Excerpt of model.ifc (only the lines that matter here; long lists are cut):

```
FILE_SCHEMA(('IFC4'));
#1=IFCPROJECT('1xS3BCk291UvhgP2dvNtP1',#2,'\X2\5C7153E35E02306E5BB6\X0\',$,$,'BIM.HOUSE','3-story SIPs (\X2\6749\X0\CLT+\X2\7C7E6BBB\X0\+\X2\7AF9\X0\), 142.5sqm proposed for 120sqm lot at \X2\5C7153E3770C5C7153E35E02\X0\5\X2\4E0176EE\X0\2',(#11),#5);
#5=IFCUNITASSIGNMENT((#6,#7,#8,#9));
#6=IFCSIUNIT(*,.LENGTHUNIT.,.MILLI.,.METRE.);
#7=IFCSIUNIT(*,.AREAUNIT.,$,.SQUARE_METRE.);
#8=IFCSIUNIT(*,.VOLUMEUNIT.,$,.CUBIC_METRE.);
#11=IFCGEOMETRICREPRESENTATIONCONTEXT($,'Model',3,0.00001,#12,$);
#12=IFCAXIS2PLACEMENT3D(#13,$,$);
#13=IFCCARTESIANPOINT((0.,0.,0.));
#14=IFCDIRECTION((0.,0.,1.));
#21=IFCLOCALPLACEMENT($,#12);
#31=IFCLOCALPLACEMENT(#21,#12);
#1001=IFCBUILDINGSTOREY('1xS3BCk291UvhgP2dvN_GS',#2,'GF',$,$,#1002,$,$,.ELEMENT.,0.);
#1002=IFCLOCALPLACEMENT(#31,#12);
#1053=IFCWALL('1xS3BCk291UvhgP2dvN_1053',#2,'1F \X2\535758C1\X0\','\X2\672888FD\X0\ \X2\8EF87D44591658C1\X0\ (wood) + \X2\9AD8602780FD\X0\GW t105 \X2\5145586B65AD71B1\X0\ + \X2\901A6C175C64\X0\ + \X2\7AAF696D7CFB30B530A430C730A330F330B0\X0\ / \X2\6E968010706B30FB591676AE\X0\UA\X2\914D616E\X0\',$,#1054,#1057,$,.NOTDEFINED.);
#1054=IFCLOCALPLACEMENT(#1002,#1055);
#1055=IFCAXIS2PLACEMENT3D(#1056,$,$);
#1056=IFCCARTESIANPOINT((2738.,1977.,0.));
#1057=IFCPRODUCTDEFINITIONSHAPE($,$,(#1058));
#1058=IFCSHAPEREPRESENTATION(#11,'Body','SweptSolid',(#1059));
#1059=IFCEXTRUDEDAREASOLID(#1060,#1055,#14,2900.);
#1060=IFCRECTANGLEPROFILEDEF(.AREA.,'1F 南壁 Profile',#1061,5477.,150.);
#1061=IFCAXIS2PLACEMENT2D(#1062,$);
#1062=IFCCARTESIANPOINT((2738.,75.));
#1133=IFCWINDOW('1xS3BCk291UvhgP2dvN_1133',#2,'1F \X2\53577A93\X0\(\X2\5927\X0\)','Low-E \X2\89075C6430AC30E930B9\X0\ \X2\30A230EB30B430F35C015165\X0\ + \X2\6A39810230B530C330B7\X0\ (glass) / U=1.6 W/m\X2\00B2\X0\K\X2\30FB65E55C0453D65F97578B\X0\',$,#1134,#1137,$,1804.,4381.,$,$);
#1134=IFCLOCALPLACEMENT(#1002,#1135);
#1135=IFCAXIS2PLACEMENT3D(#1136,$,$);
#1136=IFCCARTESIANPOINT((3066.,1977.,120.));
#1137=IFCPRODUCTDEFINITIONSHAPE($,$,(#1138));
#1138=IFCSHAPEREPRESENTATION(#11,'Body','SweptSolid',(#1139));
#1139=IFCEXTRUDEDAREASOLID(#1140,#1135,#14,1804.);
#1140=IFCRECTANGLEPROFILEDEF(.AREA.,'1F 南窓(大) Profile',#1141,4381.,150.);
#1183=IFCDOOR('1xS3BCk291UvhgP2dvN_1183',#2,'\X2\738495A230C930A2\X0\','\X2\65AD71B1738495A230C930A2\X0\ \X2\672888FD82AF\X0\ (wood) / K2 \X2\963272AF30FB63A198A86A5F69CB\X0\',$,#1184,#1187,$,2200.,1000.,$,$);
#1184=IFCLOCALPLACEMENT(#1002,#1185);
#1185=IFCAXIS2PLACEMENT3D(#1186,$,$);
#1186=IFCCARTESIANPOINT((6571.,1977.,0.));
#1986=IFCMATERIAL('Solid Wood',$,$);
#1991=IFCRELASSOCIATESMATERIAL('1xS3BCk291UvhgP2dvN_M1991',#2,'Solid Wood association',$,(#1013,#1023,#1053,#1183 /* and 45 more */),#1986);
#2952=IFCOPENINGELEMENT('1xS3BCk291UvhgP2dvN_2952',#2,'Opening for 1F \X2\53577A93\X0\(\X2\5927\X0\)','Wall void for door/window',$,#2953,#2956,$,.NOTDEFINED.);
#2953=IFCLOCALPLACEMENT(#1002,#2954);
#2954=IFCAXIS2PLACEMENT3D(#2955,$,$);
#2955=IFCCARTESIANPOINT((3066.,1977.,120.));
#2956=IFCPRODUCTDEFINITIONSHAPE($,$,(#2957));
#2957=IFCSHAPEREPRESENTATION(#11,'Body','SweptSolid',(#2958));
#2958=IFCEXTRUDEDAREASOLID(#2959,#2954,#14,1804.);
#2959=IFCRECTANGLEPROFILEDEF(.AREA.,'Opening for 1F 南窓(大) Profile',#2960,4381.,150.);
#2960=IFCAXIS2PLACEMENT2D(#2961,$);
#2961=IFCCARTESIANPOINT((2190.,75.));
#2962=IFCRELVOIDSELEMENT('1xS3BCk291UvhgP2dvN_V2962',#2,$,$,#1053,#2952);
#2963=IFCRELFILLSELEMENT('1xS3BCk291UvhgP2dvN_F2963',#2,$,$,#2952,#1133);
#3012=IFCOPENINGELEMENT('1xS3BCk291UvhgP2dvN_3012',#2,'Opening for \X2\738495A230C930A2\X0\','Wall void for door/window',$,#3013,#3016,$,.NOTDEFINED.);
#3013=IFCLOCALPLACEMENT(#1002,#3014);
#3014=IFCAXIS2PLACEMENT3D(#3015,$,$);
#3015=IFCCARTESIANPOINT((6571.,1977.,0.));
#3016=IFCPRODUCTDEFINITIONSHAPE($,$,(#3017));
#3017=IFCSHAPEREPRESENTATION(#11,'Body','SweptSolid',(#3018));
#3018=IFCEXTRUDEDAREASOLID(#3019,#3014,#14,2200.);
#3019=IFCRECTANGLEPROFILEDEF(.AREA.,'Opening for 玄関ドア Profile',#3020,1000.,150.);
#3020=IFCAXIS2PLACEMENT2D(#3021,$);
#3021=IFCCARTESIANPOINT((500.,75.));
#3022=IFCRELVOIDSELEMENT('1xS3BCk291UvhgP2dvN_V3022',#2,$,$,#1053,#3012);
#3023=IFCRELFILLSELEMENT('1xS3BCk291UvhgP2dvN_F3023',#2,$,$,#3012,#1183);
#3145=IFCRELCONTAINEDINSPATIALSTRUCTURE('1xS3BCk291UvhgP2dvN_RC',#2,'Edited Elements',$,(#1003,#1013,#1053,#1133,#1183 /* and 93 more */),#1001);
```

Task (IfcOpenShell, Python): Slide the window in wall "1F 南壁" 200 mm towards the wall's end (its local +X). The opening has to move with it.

```python
import ifcopenshell
import ifcopenshell.api.geometry
import ifcopenshell.util.placement

model = ifcopenshell.open("model.ifc")

window = model.by_id(1133)
opening = window.FillsVoids[0].RelatingOpeningElement
wall = opening.VoidsElements[0].RelatingBuildingElement

wall_matrix = ifcopenshell.util.placement.get_local_placement(wall.ObjectPlacement)
shift = wall_matrix[:3, 0] * 200.0
before = ifcopenshell.util.placement.get_local_placement(window.ObjectPlacement)[:3, 3].copy()

# The window is not placed relative to its opening, so move both.
for product in (opening, window):
    matrix = ifcopenshell.util.placement.get_local_placement(product.ObjectPlacement)
    matrix[:3, 3] += shift
    ifcopenshell.api.geometry.edit_object_placement(model, product=product, matrix=matrix, is_si=False)

after = ifcopenshell.util.placement.get_local_placement(window.ObjectPlacement)[:3, 3]
print("window moved by", (after - before).round(3) + 0.0)

model.write("model_rev.ifc")
```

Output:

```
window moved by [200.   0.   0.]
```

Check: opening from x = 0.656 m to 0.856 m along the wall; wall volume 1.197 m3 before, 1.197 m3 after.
